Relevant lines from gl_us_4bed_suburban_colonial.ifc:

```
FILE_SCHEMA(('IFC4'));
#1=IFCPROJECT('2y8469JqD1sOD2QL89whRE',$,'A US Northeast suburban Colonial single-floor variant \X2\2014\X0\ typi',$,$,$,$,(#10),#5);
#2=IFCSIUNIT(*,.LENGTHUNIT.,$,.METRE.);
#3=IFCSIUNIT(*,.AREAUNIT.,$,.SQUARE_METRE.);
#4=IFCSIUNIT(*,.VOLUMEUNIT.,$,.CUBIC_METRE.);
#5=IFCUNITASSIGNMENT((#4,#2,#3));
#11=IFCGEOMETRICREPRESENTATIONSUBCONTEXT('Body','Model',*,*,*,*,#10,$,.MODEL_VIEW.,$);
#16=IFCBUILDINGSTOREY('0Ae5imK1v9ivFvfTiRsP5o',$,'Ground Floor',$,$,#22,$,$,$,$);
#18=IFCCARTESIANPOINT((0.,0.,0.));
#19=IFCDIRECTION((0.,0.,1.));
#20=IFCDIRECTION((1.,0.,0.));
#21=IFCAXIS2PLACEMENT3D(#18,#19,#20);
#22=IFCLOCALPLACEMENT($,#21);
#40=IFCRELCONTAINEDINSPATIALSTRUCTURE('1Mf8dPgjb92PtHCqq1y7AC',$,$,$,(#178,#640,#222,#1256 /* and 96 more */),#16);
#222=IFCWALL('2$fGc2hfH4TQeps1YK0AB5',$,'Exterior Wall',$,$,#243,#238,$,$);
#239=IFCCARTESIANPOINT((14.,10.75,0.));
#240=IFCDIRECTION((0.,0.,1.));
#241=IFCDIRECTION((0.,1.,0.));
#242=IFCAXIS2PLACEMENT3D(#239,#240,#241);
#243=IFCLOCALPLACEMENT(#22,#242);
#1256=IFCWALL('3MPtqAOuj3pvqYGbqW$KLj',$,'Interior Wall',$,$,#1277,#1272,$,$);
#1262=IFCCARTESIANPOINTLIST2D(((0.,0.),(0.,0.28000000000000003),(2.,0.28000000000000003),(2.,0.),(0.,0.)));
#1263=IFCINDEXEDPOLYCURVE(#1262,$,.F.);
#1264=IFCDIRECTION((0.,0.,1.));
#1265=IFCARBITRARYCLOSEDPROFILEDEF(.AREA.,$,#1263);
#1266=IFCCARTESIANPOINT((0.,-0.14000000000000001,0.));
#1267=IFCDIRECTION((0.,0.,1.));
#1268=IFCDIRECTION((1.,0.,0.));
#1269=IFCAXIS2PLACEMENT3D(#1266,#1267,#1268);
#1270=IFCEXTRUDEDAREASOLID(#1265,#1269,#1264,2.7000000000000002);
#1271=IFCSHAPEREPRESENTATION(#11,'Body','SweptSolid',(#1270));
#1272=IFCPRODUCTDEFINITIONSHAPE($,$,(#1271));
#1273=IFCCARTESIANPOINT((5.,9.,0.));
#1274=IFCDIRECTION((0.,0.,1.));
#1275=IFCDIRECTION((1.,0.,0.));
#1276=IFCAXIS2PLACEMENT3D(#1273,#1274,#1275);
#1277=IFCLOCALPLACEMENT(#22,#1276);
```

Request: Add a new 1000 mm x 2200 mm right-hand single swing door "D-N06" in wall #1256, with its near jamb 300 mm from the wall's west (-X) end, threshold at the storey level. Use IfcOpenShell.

```python
import numpy as np
import ifcopenshell
import ifcopenshell.api.feature
import ifcopenshell.api.geometry
import ifcopenshell.api.root
import ifcopenshell.api.spatial
import ifcopenshell.geom
import ifcopenshell.util.element
import ifcopenshell.util.placement
import ifcopenshell.util.representation
import ifcopenshell.util.shape
import ifcopenshell.util.unit

model = ifcopenshell.open("gl_us_4bed_suburban_colonial.ifc")
unit_scale = ifcopenshell.util.unit.calculate_unit_scale(model)
settings = ifcopenshell.geom.settings()


def volume(element):
    """Net volume in cubic metres, openings subtracted."""
    shape = ifcopenshell.geom.create_shape(settings, element)
    return ifcopenshell.util.shape.get_volume(shape.geometry)


wall = model.by_id(1256)
storey = ifcopenshell.util.element.get_container(wall, ifc_class="IfcBuildingStorey")
context = ifcopenshell.util.representation.get_context(model, "Model", "Body", "MODEL_VIEW")
before = volume(wall)

width, height, from_end, sill = 1, 2.2, 0.3, 0.0  # metres

# The wall runs along its own X axis, and the end named is its -X end.
wall_shape = ifcopenshell.geom.create_shape(settings, wall)
x, y, z = ifcopenshell.util.shape.get_vertices(wall_shape.geometry).T
start = x.min() + from_end
face, thickness = float(y.min()), float(y.max() - y.min())
wall_matrix = ifcopenshell.util.placement.get_local_placement(wall.ObjectPlacement)
level = ifcopenshell.util.placement.get_local_placement(storey.ObjectPlacement)[2, 3]


def in_wall(x, y):
    """Placement at x, y metres in the wall's axes, at sill height."""
    matrix = wall_matrix.copy()
    matrix[:, 3] = wall_matrix @ np.array([x / unit_scale, y / unit_scale, 0.0, 1.0])
    matrix[2, 3] = level + sill / unit_scale
    return matrix


# Opening: a box that overshoots both wall faces by 50 mm.
opening = ifcopenshell.api.root.create_entity(model, ifc_class="IfcOpeningElement", predefined_type="OPENING")
box = ifcopenshell.api.geometry.add_wall_representation(
    model, context=context, length=width, height=height, thickness=thickness + 0.1
)
ifcopenshell.api.geometry.assign_representation(model, product=opening, representation=box)
ifcopenshell.api.geometry.edit_object_placement(model, product=opening, matrix=in_wall(start, face - 0.05), is_si=False)
ifcopenshell.api.feature.add_feature(model, feature=opening, element=wall)

door = ifcopenshell.api.root.create_entity(model, ifc_class="IfcDoor", name="D-N06", predefined_type="DOOR")
door.OverallWidth, door.OverallHeight = width / unit_scale, height / unit_scale
door.OperationType = "SINGLE_SWING_RIGHT"
body = ifcopenshell.api.geometry.add_door_representation(
    model,
    context=context,
    overall_width=door.OverallWidth,
    overall_height=door.OverallHeight,
    operation_type="SINGLE_SWING_RIGHT",
    lining_properties={"LiningDepth": thickness / unit_scale, "ThresholdDepth": thickness / unit_scale},
)
ifcopenshell.api.geometry.assign_representation(model, product=door, representation=body)
ifcopenshell.api.spatial.assign_container(model, products=[door], relating_structure=storey)
ifcopenshell.api.feature.add_filling(model, opening=opening, element=door)

# The lining spans the wall, so the door starts at the wall face.
ifcopenshell.api.geometry.edit_object_placement(model, product=door, matrix=in_wall(start, face), is_si=False)

after = volume(wall)

print(f"wall volume {before:.3f} -> {after:.3f} m3")

model.write("gl_us_4bed_suburban_colonial_v2.ifc")
```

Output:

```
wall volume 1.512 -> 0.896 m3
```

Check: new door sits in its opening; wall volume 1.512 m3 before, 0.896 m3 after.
